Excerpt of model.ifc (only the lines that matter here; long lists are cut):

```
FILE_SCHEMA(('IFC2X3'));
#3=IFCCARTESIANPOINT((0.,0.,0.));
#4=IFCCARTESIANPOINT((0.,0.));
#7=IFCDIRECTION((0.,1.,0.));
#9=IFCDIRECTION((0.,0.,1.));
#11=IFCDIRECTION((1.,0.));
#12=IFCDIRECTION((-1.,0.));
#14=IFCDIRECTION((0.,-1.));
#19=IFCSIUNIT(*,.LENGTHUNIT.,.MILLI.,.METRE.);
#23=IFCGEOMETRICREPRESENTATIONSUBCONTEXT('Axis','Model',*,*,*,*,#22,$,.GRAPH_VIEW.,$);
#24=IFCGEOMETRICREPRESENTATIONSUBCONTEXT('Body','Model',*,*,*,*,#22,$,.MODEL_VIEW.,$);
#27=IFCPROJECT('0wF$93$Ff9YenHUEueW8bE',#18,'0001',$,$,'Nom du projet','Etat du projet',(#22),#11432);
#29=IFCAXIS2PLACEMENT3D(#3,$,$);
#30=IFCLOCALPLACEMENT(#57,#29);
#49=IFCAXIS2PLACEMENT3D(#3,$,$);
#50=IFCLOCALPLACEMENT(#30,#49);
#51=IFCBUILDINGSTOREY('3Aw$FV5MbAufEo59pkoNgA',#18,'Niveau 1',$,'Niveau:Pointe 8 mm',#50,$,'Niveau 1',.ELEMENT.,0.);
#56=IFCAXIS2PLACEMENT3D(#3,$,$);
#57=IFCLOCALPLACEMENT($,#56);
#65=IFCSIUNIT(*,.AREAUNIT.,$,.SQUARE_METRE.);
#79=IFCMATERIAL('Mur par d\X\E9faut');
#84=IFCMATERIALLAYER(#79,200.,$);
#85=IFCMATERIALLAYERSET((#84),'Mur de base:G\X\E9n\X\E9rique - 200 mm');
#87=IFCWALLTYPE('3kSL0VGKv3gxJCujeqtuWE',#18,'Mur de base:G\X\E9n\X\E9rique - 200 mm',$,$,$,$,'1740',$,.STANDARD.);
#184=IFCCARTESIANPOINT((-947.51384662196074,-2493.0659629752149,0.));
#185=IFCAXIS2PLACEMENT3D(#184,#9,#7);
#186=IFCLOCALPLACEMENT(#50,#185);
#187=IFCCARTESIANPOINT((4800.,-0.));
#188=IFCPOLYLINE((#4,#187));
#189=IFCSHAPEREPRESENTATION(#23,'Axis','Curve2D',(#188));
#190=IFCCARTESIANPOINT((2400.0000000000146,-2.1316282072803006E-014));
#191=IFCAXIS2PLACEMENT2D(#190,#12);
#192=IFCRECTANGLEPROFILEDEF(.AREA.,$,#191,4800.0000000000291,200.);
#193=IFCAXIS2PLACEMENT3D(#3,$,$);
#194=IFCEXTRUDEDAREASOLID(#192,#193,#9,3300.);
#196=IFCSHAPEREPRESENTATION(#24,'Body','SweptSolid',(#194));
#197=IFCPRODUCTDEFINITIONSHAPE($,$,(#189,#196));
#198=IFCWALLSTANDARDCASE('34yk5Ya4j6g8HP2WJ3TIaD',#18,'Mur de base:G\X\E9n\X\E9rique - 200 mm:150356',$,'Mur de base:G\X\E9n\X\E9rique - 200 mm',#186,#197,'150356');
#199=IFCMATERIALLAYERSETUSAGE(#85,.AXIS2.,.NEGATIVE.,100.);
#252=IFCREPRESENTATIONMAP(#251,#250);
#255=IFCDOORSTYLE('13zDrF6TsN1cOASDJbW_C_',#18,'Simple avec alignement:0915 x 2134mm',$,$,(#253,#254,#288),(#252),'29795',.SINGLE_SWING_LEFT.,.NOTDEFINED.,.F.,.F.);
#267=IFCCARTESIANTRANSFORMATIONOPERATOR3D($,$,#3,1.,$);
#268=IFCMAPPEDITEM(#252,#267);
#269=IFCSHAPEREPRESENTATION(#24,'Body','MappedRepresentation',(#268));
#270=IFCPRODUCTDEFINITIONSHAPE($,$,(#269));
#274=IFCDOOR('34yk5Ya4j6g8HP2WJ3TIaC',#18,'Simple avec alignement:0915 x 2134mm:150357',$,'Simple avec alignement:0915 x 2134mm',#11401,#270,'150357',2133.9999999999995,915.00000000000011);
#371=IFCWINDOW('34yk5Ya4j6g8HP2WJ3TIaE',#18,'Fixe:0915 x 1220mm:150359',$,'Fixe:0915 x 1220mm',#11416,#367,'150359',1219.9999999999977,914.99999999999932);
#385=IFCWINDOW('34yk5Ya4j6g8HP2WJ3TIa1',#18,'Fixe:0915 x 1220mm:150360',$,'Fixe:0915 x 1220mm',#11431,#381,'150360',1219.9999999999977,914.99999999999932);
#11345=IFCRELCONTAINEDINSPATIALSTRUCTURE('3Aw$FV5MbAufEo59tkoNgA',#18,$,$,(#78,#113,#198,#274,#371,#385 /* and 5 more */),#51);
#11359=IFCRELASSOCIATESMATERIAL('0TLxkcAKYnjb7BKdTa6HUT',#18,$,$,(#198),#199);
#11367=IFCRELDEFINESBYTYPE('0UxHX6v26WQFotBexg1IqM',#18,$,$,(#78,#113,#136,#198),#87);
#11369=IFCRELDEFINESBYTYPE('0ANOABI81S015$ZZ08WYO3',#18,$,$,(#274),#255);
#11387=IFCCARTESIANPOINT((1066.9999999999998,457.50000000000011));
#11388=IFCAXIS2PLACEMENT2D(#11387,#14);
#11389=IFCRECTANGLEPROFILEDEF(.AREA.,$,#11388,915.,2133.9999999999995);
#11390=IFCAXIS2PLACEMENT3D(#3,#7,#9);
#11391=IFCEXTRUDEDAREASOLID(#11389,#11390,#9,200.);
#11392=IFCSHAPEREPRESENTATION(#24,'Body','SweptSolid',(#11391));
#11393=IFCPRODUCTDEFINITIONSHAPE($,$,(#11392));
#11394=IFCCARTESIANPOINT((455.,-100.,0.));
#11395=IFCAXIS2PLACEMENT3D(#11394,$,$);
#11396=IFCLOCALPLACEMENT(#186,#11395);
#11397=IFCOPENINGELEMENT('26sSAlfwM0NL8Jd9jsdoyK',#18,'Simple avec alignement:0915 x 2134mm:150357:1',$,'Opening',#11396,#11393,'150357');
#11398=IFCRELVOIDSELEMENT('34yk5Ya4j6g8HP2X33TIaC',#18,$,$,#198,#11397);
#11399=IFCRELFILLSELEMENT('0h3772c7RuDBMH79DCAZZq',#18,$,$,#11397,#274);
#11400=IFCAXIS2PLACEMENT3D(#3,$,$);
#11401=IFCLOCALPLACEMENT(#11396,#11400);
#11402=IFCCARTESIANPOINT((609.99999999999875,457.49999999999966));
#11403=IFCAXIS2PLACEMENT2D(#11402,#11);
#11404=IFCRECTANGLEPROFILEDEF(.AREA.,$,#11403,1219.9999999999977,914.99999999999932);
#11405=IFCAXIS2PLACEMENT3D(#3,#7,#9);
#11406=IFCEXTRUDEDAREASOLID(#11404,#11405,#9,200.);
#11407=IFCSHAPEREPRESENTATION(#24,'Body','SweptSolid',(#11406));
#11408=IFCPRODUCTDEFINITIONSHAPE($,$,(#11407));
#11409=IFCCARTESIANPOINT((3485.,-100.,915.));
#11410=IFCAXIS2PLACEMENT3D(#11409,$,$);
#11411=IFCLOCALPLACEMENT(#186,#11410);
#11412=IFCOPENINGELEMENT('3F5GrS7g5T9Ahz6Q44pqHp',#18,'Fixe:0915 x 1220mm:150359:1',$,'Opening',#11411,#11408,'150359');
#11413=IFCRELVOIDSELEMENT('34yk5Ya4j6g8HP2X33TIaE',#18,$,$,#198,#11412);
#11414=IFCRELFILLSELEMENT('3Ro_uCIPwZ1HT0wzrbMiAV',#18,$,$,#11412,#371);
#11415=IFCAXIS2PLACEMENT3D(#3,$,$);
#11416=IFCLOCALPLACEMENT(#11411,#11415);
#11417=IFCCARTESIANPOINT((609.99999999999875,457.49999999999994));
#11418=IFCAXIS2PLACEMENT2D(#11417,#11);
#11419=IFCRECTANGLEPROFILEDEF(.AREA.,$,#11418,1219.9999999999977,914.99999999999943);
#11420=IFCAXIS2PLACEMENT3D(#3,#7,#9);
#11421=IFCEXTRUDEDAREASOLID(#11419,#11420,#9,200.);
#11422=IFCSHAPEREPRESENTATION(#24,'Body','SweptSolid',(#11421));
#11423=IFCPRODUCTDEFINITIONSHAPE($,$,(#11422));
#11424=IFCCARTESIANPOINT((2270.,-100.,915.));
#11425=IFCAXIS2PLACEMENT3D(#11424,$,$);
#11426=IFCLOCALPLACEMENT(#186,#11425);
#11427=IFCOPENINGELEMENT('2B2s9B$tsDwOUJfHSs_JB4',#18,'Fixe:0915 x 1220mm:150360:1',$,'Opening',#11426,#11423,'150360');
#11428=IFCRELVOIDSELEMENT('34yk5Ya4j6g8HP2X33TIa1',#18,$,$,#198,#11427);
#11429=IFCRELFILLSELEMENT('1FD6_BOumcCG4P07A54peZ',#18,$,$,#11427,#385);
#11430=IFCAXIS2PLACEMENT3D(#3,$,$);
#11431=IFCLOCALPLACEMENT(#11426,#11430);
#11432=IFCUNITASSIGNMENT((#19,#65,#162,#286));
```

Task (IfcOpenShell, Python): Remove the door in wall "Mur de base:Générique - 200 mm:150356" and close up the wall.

```python
import ifcopenshell
import ifcopenshell.api.feature
import ifcopenshell.api.root
import ifcopenshell.geom
import ifcopenshell.util.shape

model = ifcopenshell.open("model.ifc")
settings = ifcopenshell.geom.settings()


def volume(element):
    """Net volume in cubic metres, openings subtracted."""
    shape = ifcopenshell.geom.create_shape(settings, element)
    return ifcopenshell.util.shape.get_volume(shape.geometry)


door = model.by_guid("34yk5Ya4j6g8HP2WJ3TIaC")
opening = door.FillsVoids[0].RelatingOpeningElement
wall = opening.VoidsElements[0].RelatingBuildingElement
before = volume(wall)

ifcopenshell.api.root.remove_product(model, product=door)
ifcopenshell.api.feature.remove_feature(model, feature=opening)

after = volume(wall)

print(f"wall volume {before:.3f} -> {after:.3f} m3")

model.write("model_updated.ifc")
```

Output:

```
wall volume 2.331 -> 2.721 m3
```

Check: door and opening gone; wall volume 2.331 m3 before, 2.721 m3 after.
